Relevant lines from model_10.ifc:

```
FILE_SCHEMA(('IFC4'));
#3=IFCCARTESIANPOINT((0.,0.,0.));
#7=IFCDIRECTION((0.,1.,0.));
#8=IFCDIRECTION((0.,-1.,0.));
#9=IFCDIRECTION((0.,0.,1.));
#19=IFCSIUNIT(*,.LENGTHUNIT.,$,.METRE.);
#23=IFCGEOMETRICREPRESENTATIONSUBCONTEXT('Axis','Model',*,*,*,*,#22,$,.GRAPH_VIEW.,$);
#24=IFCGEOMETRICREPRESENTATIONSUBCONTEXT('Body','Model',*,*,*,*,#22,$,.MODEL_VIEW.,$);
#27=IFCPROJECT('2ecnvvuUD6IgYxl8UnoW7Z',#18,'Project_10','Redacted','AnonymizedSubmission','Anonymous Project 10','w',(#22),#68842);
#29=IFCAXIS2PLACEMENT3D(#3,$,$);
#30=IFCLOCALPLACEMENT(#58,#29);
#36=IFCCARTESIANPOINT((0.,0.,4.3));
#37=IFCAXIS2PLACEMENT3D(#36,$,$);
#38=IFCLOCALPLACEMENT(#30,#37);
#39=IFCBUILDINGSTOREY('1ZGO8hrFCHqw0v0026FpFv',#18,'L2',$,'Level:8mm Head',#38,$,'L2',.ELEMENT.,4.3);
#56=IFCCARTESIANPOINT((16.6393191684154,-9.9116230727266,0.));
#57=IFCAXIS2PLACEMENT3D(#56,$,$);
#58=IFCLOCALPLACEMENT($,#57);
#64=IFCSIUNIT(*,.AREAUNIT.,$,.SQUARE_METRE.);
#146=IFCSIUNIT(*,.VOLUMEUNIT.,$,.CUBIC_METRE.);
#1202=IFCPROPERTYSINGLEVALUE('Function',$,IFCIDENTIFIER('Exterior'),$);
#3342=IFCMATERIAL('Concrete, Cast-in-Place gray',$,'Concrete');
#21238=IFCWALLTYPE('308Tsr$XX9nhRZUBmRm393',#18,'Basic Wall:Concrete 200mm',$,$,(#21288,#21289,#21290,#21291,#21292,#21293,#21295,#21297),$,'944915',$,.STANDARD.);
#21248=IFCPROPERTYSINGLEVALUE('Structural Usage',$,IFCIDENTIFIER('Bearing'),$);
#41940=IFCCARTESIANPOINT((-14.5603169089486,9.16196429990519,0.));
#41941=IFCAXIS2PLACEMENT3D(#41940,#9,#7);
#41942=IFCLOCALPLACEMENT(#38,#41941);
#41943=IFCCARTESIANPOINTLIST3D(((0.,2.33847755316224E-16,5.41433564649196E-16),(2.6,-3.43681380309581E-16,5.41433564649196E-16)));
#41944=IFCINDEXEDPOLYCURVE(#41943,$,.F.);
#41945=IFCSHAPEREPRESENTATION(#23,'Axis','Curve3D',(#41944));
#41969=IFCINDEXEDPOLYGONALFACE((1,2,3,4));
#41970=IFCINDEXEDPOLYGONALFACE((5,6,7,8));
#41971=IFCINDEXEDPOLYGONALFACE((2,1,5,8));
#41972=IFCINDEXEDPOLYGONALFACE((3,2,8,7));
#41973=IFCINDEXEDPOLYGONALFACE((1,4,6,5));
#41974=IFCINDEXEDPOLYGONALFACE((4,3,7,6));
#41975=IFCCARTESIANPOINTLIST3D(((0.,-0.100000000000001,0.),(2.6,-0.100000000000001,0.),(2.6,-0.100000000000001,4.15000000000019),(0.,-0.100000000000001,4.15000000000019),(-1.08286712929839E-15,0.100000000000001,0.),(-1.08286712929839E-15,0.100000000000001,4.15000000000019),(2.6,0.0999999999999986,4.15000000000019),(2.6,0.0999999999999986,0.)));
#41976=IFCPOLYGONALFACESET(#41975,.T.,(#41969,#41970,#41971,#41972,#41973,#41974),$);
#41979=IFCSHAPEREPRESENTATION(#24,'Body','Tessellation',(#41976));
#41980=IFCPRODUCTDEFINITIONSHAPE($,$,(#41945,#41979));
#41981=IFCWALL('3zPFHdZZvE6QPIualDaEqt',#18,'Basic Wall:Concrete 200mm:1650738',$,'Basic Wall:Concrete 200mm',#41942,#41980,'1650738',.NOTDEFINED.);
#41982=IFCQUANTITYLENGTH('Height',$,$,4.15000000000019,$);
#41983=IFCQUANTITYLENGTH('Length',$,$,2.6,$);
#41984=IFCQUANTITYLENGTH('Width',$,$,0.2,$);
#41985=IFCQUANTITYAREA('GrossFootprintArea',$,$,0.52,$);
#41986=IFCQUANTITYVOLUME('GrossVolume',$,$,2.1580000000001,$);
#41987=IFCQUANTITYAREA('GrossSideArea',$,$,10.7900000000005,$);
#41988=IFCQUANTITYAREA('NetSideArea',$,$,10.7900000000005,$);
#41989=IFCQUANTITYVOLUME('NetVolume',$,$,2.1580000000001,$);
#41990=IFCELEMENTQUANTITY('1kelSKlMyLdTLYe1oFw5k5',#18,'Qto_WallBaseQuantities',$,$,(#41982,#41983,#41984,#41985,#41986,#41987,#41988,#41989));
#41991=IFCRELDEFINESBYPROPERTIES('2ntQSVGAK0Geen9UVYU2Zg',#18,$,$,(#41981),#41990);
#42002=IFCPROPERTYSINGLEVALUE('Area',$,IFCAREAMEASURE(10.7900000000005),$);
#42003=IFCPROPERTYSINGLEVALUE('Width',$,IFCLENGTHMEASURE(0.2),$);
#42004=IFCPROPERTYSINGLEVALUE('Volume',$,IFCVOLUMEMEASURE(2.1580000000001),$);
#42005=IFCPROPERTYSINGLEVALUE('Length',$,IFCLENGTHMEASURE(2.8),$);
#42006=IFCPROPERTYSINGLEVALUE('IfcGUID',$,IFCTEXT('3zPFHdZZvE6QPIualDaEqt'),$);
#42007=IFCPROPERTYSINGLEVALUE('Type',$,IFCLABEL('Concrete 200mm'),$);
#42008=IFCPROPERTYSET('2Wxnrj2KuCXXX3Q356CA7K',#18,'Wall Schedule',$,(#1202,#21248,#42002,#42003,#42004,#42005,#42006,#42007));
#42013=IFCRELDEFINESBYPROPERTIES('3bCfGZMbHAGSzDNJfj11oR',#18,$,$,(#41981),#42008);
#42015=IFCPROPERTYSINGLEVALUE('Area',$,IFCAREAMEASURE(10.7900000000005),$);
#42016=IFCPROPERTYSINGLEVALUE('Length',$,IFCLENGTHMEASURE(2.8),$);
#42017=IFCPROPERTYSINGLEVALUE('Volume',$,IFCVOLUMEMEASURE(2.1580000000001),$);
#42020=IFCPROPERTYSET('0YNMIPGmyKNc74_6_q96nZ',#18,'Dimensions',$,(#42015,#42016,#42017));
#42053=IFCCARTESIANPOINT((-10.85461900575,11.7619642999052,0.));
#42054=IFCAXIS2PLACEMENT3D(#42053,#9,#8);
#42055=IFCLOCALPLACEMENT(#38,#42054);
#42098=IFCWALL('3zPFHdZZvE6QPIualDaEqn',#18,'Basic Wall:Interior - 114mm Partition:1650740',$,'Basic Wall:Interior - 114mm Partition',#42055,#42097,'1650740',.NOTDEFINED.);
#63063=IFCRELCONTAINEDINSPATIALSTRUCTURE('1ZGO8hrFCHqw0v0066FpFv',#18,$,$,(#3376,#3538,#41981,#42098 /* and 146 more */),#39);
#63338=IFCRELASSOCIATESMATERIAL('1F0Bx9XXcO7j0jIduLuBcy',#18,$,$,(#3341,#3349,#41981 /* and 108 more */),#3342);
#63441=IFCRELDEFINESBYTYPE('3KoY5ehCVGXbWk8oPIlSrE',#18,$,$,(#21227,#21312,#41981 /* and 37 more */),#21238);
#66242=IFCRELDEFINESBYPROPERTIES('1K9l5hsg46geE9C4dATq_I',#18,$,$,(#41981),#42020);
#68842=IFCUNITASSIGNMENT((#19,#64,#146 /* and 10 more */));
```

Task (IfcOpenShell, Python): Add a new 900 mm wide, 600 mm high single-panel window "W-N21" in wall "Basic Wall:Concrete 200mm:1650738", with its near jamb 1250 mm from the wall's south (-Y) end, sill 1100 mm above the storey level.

```python
import numpy as np
import ifcopenshell
import ifcopenshell.api.feature
import ifcopenshell.api.geometry
import ifcopenshell.api.pset
import ifcopenshell.api.root
import ifcopenshell.api.spatial
import ifcopenshell.geom
import ifcopenshell.util.element
import ifcopenshell.util.placement
import ifcopenshell.util.representation
import ifcopenshell.util.shape
import ifcopenshell.util.unit

model = ifcopenshell.open("model_10.ifc")
unit_scale = ifcopenshell.util.unit.calculate_unit_scale(model)
area_scale = ifcopenshell.util.unit.calculate_unit_scale(model, "AREAUNIT")
volume_scale = ifcopenshell.util.unit.calculate_unit_scale(model, "VOLUMEUNIT")
settings = ifcopenshell.geom.settings()


def volume(element):
    """Net volume in cubic metres, openings subtracted."""
    shape = ifcopenshell.geom.create_shape(settings, element)
    return ifcopenshell.util.shape.get_volume(shape.geometry)


wall = model.by_id(41981)
storey = ifcopenshell.util.element.get_container(wall, ifc_class="IfcBuildingStorey")
context = ifcopenshell.util.representation.get_context(model, "Model", "Body", "MODEL_VIEW")
before = volume(wall)

width, height, from_end, sill = 0.9, 0.6, 1.25, 1.1  # metres

# The wall runs along its own X axis, and the end named is its -X end.
wall_shape = ifcopenshell.geom.create_shape(settings, wall)
x, y, z = ifcopenshell.util.shape.get_vertices(wall_shape.geometry).T
start = x.min() + from_end
face, thickness = float(y.min()), float(y.max() - y.min())
wall_matrix = ifcopenshell.util.placement.get_local_placement(wall.ObjectPlacement)
level = ifcopenshell.util.placement.get_local_placement(storey.ObjectPlacement)[2, 3]


def in_wall(x, y):
    """Placement at x, y metres in the wall's axes, at sill height."""
    matrix = wall_matrix.copy()
    matrix[:, 3] = wall_matrix @ np.array([x / unit_scale, y / unit_scale, 0.0, 1.0])
    matrix[2, 3] = level + sill / unit_scale
    return matrix


# Opening: a box that overshoots both wall faces by 50 mm.
opening = ifcopenshell.api.root.create_entity(model, ifc_class="IfcOpeningElement", predefined_type="OPENING")
box = ifcopenshell.api.geometry.add_wall_representation(
    model, context=context, length=width, height=height, thickness=thickness + 0.1
)
ifcopenshell.api.geometry.assign_representation(model, product=opening, representation=box)
ifcopenshell.api.geometry.edit_object_placement(model, product=opening, matrix=in_wall(start, face - 0.05), is_si=False)
ifcopenshell.api.feature.add_feature(model, feature=opening, element=wall)

window = ifcopenshell.api.root.create_entity(model, ifc_class="IfcWindow", name="W-N21", predefined_type="WINDOW")
window.OverallWidth, window.OverallHeight = width / unit_scale, height / unit_scale
window.PartitioningType = "SINGLE_PANEL"
body = ifcopenshell.api.geometry.add_window_representation(
    model,
    context=context,
    overall_width=window.OverallWidth,
    overall_height=window.OverallHeight,
    partition_type="SINGLE_PANEL",
)
ifcopenshell.api.geometry.assign_representation(model, product=window, representation=body)
ifcopenshell.api.spatial.assign_container(model, products=[window], relating_structure=storey)
ifcopenshell.api.feature.add_filling(model, opening=opening, element=window)

# Centre the window in the wall's thickness.
ifcopenshell.api.geometry.edit_object_placement(model, product=window, matrix=in_wall(start, face), is_si=False)
window_shape = ifcopenshell.geom.create_shape(settings, window)
depth = ifcopenshell.util.shape.get_vertices(window_shape.geometry)[:, 1]
offset = face + thickness / 2 - (depth.min() + depth.max()) / 2
ifcopenshell.api.geometry.edit_object_placement(model, product=window, matrix=in_wall(start, offset), is_si=False)

after = volume(wall)

# Update the wall's stored quantities.
qto = model.by_id(ifcopenshell.util.element.get_pset(wall, "Qto_WallBaseQuantities", should_inherit=False)["id"])
ifcopenshell.api.pset.edit_qto(model, qto=qto, properties={
    "NetSideArea": after / thickness / area_scale,
    "NetVolume": after / volume_scale,
})
pset = model.by_id(ifcopenshell.util.element.get_pset(wall, "Wall Schedule", should_inherit=False)["id"])
ifcopenshell.api.pset.edit_pset(model, pset=pset, properties={
    "Area": model.create_entity("IfcAreaMeasure", after / thickness / area_scale),
    "Volume": model.create_entity("IfcVolumeMeasure", after / volume_scale),
})
pset = model.by_id(ifcopenshell.util.element.get_pset(wall, "Dimensions", should_inherit=False)["id"])
ifcopenshell.api.pset.edit_pset(model, pset=pset, properties={
    "Area": model.create_entity("IfcAreaMeasure", after / thickness / area_scale),
    "Volume": model.create_entity("IfcVolumeMeasure", after / volume_scale),
})

print(f"wall volume {before:.3f} -> {after:.3f} m3")

model.write("model_10_v2.ifc")
```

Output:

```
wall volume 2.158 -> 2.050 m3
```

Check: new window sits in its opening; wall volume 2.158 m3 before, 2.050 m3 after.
